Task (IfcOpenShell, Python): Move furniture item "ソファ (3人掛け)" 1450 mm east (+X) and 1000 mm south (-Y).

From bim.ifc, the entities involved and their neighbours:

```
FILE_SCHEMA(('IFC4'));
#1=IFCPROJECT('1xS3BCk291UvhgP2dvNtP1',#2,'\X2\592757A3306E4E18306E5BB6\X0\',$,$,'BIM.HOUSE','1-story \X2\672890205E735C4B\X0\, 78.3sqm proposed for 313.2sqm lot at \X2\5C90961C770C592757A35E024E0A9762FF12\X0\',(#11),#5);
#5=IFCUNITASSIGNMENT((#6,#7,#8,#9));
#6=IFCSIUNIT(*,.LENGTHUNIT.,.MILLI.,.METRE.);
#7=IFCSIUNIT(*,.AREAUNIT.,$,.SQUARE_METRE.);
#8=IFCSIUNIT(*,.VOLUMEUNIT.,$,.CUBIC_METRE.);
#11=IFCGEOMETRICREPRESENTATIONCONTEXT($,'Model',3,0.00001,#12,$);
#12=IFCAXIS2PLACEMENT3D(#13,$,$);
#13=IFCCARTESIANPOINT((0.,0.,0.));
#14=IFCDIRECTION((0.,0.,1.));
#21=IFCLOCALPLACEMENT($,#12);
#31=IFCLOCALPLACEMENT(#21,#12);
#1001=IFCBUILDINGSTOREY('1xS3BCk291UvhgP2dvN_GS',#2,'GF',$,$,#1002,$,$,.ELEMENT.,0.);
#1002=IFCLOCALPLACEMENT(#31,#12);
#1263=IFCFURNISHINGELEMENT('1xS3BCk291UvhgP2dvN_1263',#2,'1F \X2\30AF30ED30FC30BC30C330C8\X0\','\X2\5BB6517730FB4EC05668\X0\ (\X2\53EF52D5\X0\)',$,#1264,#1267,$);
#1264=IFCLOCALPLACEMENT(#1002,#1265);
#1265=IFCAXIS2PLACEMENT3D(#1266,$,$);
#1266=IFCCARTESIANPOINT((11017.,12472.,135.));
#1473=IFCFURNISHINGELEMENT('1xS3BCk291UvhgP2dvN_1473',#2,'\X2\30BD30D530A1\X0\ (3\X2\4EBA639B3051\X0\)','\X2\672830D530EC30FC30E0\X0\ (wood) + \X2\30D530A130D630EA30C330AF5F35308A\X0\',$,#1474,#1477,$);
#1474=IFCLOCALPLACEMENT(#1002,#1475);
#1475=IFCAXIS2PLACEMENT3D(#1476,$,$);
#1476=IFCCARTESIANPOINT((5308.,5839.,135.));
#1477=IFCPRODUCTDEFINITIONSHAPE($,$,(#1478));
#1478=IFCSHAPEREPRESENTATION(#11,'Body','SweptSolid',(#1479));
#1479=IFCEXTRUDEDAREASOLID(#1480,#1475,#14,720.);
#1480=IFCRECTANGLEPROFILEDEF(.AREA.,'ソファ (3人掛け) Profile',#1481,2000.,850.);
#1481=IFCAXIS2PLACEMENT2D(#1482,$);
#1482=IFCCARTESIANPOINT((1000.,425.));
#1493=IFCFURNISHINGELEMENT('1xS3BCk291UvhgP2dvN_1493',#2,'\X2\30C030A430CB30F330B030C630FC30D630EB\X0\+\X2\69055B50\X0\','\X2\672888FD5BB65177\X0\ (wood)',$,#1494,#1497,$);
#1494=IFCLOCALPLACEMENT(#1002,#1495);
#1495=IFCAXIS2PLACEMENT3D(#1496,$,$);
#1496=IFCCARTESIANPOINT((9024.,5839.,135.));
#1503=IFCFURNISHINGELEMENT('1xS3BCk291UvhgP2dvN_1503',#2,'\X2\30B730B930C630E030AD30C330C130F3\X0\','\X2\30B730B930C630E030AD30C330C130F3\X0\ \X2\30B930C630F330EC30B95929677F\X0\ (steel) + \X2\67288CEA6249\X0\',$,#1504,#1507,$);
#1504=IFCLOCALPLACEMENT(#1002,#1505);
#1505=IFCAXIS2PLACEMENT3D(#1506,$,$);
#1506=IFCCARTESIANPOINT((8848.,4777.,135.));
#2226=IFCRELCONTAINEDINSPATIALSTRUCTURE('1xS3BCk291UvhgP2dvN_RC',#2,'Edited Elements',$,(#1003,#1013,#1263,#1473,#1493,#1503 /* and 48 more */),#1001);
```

```python
import ifcopenshell
import ifcopenshell.api.geometry
import ifcopenshell.util.placement
import ifcopenshell.util.unit

model = ifcopenshell.open("bim.ifc")
unit_scale = ifcopenshell.util.unit.calculate_unit_scale(model)

item = model.by_guid("1xS3BCk291UvhgP2dvN_1473")
matrix = ifcopenshell.util.placement.get_local_placement(item.ObjectPlacement)
matrix[0, 3] += 1.45 / unit_scale
matrix[1, 3] -= 1 / unit_scale
ifcopenshell.api.geometry.edit_object_placement(model, product=item, matrix=matrix, is_si=False)

print(ifcopenshell.util.placement.get_local_placement(item.ObjectPlacement).round(3) + 0.0)

model.write("bim-out.ifc")
```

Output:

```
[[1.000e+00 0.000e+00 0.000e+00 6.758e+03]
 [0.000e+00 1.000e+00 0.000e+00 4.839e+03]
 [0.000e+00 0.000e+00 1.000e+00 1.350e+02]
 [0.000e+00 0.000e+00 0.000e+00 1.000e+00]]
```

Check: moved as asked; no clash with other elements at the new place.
